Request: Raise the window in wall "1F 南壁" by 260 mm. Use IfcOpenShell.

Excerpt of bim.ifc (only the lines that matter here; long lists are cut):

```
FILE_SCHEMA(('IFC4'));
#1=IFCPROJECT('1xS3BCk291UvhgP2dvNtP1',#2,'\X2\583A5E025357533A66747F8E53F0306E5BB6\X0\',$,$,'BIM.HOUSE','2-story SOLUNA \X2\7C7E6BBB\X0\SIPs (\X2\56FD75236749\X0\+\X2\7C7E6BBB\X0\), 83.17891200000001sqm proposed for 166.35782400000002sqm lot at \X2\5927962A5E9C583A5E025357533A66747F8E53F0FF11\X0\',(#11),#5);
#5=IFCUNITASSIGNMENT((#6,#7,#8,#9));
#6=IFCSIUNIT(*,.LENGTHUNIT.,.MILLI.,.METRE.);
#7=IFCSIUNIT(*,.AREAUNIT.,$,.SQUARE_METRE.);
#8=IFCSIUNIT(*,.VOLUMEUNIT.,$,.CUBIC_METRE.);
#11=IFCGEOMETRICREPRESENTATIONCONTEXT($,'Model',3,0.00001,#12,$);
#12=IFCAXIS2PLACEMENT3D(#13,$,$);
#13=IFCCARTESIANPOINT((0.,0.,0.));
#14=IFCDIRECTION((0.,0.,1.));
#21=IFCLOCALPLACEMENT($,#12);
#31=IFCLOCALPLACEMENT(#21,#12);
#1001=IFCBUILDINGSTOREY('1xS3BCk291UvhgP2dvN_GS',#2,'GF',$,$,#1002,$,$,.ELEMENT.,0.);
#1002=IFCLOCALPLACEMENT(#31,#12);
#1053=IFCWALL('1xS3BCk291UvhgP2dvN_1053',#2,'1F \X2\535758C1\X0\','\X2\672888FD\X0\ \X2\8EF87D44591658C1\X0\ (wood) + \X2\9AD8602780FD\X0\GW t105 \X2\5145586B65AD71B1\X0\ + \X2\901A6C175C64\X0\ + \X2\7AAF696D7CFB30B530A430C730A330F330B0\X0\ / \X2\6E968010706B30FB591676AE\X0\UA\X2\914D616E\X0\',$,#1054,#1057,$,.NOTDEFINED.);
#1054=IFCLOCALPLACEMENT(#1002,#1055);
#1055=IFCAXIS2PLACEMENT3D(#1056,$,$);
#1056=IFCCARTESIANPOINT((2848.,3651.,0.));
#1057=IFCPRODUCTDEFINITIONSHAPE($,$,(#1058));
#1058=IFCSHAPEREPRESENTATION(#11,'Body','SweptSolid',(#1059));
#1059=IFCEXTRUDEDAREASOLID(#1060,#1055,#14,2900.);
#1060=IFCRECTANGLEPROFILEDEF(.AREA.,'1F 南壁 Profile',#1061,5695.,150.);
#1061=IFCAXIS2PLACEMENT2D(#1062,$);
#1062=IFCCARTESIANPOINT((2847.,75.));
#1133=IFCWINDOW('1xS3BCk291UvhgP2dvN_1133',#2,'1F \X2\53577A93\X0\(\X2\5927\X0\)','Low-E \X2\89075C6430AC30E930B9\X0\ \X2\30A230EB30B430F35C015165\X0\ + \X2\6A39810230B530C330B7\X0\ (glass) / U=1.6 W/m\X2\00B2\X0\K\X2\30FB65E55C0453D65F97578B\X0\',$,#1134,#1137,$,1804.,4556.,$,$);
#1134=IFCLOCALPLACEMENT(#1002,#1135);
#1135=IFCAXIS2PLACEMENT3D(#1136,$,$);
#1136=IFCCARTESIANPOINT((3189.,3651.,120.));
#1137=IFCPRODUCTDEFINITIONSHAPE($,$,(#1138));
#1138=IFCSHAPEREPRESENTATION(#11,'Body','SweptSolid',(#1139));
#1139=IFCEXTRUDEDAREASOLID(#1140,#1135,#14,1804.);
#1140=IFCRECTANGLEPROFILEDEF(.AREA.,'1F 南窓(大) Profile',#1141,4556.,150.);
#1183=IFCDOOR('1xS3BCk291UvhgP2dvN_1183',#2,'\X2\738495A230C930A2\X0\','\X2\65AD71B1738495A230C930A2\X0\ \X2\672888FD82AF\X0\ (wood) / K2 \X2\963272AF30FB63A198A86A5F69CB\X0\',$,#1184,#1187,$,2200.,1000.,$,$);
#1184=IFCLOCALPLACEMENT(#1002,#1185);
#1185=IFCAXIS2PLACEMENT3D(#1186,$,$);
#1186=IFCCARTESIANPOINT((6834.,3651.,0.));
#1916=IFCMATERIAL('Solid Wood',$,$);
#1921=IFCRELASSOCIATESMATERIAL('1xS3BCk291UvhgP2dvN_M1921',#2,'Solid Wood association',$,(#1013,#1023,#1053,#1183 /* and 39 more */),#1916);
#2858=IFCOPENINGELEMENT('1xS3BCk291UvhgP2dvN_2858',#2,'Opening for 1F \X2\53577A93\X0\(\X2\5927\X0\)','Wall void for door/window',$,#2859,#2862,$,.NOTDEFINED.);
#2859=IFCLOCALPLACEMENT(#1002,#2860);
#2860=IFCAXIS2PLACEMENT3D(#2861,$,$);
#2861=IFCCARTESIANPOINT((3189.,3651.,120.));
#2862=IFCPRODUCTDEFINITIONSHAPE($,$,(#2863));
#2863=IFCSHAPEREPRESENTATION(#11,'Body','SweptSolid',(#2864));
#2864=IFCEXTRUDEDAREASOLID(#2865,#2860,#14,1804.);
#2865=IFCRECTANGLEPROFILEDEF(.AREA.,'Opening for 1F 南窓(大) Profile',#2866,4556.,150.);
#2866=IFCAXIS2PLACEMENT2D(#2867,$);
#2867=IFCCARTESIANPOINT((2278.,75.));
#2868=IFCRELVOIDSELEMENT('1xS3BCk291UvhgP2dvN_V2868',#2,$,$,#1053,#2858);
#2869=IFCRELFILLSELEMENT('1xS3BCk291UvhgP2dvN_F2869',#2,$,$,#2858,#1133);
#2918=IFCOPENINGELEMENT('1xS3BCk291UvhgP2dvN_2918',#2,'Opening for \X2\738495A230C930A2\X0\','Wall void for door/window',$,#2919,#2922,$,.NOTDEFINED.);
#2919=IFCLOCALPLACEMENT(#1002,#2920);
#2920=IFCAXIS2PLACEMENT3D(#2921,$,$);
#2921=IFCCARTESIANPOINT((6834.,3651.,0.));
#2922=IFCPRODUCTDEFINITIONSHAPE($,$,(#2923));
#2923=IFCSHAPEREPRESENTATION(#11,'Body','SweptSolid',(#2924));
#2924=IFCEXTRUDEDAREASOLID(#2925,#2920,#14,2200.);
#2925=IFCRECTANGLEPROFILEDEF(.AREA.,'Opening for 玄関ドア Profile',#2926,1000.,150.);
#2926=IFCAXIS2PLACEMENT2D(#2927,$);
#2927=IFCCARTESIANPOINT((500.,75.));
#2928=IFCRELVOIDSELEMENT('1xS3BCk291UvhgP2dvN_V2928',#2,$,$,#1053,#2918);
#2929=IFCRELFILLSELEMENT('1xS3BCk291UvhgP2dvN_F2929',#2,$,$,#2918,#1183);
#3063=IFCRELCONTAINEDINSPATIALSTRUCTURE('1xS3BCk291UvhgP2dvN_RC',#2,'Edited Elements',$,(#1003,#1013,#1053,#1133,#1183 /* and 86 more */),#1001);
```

```python
import numpy as np
import ifcopenshell
import ifcopenshell.api.geometry
import ifcopenshell.util.placement
import ifcopenshell.util.unit

model = ifcopenshell.open("bim.ifc")
unit_scale = ifcopenshell.util.unit.calculate_unit_scale(model)

window = model.by_guid("1xS3BCk291UvhgP2dvN_1133")
opening = window.FillsVoids[0].RelatingOpeningElement
dz = 260.0

shift = np.array([0.0, 0.0, dz])
# The window is not placed relative to its opening, so move both.
for product in (opening, window):
    matrix = ifcopenshell.util.placement.get_local_placement(product.ObjectPlacement)
    matrix[:3, 3] += shift
    ifcopenshell.api.geometry.edit_object_placement(model, product=product, matrix=matrix, is_si=False)

print(f"moved by {dz * unit_scale:+.3f} m")

model.write("bim-out.ifc")
```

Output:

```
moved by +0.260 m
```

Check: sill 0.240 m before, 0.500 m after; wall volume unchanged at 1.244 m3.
